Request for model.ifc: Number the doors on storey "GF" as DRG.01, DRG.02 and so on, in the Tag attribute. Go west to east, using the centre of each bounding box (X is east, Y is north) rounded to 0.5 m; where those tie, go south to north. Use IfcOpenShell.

First a look at what the model holds.

```python
import ifcopenshell
import ifcopenshell.util.element
import ifcopenshell.util.placement

model = ifcopenshell.open("model.ifc")
print(model.schema)
storey = next(s for s in model.by_type("IfcBuildingStorey") if s.Name == "GF")
doors = [e for e in ifcopenshell.util.element.get_decomposition(storey) if e.is_a("IfcDoor")]
for e in sorted(doors, key=lambda e: e.id()):
    origin = ifcopenshell.util.placement.get_local_placement(e.ObjectPlacement)[:3, 3]
    print(e.id(), e.Tag, e.Name, origin.round(2) + 0.0, sep=" | ")
```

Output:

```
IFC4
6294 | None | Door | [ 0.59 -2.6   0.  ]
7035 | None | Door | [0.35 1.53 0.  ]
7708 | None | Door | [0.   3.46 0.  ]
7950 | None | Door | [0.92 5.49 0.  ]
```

```python
import ifcopenshell
import ifcopenshell.geom
import ifcopenshell.util.element
import ifcopenshell.util.shape

model = ifcopenshell.open("model.ifc")
settings = ifcopenshell.geom.settings()
settings.set("use-world-coords", True)


def centre(element):
    shape = ifcopenshell.geom.create_shape(settings, element)
    return ifcopenshell.util.shape.get_bbox_centroid(shape.geometry)


storey = next(s for s in model.by_type("IfcBuildingStorey") if s.Name == "GF")
doors = [e for e in ifcopenshell.util.element.get_decomposition(storey) if e.is_a("IfcDoor")]

# Insertion points can sit at a corner or the storey origin, so sort by the geometry (in metres).
centres = {e: centre(e) for e in doors}
doors.sort(key=lambda e: (round(centres[e][0] / 0.5), centres[e][1]))

for i, e in enumerate(doors, start=1):
    number = f"DRG.{i:02d}"
    e.Tag = number
    print(e.id(), number)

model.write("model_edited.ifc")
```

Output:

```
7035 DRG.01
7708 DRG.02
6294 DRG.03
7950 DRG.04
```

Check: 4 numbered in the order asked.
